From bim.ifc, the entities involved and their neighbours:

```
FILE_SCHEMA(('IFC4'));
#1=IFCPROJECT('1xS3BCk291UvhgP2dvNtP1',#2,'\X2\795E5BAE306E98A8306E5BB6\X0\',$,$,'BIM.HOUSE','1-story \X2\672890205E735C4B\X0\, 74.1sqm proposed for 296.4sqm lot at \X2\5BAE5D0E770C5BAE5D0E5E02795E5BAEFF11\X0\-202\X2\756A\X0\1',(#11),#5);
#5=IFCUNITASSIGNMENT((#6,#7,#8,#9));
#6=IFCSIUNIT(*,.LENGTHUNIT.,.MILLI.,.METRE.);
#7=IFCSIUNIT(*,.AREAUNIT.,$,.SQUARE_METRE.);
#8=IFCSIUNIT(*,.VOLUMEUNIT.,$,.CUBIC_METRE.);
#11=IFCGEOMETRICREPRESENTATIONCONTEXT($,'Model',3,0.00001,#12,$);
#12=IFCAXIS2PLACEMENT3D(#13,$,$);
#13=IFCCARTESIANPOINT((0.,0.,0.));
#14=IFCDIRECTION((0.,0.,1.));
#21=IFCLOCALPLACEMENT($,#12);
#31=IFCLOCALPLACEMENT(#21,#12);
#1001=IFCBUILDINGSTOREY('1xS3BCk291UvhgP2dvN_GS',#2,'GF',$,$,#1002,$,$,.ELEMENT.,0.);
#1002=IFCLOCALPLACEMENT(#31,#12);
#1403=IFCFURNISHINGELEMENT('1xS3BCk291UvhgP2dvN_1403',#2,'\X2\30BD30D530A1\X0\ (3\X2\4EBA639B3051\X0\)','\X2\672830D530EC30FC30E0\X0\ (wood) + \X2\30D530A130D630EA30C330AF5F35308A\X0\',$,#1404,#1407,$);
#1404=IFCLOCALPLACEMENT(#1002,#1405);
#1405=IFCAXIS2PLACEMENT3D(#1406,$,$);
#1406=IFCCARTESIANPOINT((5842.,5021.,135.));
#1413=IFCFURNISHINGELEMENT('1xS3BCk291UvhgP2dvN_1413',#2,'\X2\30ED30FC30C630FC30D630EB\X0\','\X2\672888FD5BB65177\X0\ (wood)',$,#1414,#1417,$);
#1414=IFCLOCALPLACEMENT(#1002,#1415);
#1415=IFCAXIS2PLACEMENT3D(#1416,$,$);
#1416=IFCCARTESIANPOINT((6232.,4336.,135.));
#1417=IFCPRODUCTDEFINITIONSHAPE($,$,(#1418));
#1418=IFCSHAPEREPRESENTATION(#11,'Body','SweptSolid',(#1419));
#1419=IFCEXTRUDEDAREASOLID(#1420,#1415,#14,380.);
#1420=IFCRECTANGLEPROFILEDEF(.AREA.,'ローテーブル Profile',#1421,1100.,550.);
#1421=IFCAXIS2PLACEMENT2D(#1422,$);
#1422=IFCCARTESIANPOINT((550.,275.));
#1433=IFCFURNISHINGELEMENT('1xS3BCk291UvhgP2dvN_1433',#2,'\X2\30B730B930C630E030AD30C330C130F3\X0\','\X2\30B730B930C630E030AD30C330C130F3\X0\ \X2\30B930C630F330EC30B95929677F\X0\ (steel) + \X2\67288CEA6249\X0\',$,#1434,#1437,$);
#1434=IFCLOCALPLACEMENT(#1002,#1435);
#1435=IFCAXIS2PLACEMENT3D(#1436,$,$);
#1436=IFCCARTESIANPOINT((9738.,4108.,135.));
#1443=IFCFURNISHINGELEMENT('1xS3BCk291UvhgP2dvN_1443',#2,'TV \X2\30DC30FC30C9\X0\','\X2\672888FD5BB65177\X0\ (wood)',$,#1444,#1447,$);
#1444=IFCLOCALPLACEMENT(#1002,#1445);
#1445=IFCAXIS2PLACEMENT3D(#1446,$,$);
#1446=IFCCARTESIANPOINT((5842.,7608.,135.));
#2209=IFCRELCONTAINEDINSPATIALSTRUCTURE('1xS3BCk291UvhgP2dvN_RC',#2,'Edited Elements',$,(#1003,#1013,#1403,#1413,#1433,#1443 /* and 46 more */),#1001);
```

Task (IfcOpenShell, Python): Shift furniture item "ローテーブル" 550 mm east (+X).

```python
import ifcopenshell
import ifcopenshell.api.geometry
import ifcopenshell.util.placement

model = ifcopenshell.open("bim.ifc")

item = model.by_guid("1xS3BCk291UvhgP2dvN_1413")
matrix = ifcopenshell.util.placement.get_local_placement(item.ObjectPlacement)
matrix[0, 3] += 550.0
ifcopenshell.api.geometry.edit_object_placement(model, product=item, matrix=matrix, is_si=False)

print(ifcopenshell.util.placement.get_local_placement(item.ObjectPlacement).round(3) + 0.0)

model.write("bim_updated.ifc")
```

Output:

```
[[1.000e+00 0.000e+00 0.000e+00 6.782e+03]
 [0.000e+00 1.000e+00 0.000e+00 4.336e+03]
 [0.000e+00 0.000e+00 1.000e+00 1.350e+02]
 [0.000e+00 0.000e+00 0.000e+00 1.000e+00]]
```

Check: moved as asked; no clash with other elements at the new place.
